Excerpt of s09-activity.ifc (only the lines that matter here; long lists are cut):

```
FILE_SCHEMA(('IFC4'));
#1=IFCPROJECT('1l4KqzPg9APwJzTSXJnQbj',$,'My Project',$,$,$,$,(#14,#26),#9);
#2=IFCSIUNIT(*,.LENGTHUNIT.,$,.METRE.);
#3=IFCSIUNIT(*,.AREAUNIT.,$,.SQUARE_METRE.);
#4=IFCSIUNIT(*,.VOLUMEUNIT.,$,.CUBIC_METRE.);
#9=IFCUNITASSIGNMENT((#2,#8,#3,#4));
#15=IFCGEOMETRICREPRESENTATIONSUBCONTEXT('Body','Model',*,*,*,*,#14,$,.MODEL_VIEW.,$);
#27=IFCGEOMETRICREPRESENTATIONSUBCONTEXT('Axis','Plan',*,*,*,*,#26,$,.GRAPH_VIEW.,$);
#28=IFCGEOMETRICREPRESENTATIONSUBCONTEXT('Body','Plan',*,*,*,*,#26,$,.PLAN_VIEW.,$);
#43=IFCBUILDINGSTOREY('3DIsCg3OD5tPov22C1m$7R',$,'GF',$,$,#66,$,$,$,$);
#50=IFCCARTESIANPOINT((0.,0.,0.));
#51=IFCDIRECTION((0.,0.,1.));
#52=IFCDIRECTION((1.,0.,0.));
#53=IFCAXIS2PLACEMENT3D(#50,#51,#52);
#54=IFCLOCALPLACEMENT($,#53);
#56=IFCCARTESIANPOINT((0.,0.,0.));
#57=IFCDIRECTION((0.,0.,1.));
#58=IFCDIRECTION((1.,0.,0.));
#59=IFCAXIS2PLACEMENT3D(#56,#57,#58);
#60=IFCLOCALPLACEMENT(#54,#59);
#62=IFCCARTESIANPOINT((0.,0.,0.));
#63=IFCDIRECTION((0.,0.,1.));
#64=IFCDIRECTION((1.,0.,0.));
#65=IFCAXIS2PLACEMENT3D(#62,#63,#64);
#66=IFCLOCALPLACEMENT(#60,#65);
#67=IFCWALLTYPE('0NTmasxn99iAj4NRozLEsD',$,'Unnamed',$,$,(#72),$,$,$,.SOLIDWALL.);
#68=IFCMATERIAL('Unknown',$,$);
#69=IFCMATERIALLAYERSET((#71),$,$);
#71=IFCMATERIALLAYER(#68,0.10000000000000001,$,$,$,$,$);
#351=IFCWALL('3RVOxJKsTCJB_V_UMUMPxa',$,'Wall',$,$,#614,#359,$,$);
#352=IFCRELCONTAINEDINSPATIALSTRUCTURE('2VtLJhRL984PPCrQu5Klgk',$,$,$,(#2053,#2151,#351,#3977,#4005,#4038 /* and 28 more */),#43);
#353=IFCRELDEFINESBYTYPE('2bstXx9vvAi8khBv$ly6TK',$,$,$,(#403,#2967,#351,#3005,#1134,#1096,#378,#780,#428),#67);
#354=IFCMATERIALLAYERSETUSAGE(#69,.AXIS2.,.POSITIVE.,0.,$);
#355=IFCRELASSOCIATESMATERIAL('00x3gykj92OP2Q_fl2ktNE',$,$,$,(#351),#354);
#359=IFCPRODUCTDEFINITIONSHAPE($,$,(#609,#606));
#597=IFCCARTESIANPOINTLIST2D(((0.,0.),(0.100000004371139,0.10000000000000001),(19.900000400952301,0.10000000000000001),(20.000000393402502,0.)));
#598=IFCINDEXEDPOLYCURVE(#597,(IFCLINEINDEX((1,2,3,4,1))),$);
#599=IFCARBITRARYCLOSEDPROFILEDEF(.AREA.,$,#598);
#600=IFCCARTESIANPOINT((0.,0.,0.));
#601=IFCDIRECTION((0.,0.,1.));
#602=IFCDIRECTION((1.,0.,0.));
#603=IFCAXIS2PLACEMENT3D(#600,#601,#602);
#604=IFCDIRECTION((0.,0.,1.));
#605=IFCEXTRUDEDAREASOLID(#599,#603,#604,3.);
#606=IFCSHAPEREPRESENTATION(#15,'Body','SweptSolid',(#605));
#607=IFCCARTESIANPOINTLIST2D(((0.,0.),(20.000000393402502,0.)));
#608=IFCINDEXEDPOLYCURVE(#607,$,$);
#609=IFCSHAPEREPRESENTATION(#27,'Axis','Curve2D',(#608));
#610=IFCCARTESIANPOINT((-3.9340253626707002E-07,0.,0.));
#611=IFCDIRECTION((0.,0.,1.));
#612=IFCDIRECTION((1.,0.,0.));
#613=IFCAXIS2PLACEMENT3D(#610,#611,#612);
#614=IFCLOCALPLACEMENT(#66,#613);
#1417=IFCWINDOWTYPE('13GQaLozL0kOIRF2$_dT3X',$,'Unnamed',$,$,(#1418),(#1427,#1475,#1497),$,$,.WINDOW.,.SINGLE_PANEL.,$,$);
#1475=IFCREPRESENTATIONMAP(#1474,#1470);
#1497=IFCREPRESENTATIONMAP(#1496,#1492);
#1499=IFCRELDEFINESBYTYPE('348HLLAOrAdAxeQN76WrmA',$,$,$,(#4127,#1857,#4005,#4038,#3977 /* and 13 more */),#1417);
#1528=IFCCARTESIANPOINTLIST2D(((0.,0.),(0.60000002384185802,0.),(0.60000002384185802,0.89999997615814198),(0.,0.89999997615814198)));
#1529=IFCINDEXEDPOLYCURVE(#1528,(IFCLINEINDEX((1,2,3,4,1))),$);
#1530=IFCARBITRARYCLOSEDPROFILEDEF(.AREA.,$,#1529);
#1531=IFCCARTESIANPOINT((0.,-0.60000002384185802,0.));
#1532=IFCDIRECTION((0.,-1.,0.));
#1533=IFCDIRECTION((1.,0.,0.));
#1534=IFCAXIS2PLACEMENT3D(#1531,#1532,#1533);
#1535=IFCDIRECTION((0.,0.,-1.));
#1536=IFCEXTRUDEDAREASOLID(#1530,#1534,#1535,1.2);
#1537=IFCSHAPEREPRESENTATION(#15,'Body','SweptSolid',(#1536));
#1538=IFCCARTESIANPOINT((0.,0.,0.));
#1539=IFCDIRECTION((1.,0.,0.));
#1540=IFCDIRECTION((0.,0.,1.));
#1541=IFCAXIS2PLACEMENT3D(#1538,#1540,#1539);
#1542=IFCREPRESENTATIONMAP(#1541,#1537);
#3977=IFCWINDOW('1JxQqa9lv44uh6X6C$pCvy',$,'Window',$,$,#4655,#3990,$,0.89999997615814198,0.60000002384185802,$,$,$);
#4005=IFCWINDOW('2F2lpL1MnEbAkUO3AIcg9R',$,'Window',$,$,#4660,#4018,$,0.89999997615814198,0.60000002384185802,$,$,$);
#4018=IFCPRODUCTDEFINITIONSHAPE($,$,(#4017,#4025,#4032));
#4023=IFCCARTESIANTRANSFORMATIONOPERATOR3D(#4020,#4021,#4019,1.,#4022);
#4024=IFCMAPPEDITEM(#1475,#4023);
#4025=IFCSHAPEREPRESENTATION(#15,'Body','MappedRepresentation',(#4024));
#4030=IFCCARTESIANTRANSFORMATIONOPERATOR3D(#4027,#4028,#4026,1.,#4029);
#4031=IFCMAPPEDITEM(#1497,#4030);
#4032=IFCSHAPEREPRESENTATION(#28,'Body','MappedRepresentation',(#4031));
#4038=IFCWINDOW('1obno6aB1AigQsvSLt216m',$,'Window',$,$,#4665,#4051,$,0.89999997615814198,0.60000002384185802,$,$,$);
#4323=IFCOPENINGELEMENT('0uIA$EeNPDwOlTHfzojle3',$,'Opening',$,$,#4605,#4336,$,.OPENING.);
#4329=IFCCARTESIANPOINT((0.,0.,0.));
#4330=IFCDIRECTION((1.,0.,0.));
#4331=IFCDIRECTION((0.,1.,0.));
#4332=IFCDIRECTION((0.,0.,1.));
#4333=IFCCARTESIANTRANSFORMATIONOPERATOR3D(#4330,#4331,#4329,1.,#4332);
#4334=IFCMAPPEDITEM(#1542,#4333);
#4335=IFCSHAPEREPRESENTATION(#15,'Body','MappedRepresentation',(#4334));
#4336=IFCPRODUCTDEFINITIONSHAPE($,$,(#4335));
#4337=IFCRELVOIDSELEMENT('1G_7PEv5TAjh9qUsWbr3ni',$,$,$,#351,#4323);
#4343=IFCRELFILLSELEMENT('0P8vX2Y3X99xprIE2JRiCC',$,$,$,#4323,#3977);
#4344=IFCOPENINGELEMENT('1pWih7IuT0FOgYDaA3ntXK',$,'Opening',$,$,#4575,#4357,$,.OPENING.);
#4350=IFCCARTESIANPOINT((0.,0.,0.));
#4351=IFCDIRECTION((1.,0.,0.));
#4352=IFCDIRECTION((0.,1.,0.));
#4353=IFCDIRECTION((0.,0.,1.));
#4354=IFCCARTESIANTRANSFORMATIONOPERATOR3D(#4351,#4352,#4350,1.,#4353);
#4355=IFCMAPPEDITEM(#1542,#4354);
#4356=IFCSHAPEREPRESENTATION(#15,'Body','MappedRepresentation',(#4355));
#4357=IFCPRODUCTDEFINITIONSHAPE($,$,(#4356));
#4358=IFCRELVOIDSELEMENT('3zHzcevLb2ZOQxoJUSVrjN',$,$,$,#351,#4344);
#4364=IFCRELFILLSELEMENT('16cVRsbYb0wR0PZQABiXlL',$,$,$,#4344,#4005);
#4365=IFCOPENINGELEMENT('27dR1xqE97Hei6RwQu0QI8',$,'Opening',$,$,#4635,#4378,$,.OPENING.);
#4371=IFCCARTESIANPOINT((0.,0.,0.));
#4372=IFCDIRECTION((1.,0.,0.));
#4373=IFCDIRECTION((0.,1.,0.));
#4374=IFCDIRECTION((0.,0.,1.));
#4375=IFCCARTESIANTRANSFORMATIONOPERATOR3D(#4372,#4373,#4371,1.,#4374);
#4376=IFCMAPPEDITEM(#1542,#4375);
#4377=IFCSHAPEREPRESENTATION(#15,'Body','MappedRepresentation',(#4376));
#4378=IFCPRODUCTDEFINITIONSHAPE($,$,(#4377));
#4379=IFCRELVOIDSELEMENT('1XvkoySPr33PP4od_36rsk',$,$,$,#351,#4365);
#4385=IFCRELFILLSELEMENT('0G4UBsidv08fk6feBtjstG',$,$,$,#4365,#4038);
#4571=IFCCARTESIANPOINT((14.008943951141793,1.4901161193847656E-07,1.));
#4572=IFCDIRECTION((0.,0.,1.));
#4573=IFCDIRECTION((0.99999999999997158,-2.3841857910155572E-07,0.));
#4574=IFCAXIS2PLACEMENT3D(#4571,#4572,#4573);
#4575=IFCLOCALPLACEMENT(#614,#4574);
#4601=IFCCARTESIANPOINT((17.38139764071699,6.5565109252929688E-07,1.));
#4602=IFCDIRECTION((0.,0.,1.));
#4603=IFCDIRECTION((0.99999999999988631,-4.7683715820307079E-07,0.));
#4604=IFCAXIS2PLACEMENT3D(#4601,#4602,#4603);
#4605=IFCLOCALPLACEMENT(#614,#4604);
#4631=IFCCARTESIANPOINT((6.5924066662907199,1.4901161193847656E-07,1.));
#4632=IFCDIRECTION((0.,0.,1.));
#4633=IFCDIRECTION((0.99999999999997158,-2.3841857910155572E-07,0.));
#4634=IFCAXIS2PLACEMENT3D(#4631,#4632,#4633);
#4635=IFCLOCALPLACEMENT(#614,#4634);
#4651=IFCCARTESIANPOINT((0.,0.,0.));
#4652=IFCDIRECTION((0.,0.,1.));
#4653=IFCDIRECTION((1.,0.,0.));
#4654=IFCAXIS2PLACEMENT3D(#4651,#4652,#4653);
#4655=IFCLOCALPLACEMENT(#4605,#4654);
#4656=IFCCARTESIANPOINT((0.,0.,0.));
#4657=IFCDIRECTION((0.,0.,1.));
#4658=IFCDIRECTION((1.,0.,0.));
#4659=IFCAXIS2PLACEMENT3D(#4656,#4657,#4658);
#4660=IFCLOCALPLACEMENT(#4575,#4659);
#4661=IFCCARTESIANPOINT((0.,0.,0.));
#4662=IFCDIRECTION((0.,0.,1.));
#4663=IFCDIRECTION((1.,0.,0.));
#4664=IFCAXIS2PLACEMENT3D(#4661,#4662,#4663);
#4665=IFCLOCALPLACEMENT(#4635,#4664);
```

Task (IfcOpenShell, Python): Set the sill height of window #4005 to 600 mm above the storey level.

```python
import numpy as np
import ifcopenshell
import ifcopenshell.api.geometry
import ifcopenshell.geom
import ifcopenshell.util.element
import ifcopenshell.util.placement
import ifcopenshell.util.shape
import ifcopenshell.util.unit

model = ifcopenshell.open("s09-activity.ifc")
unit_scale = ifcopenshell.util.unit.calculate_unit_scale(model)

window = model.by_id(4005)
opening = window.FillsVoids[0].RelatingOpeningElement
storey = ifcopenshell.util.element.get_container(window, ifc_class="IfcBuildingStorey")
level = ifcopenshell.util.placement.get_local_placement(storey.ObjectPlacement)[2, 3]

# The opening's origin need not be at the sill, so measure its lowest point.
shape = ifcopenshell.geom.create_shape(ifcopenshell.geom.settings(), opening)
bottom = ifcopenshell.util.shape.get_shape_bottom_elevation(shape, shape.geometry) / unit_scale
dz = level + 0.6 - bottom

shift = np.array([0.0, 0.0, dz])
# The window is placed relative to its opening, so it follows when the opening moves.
matrix = ifcopenshell.util.placement.get_local_placement(opening.ObjectPlacement)
matrix[:3, 3] += shift
ifcopenshell.api.geometry.edit_object_placement(
    model, product=opening, matrix=matrix, is_si=False, should_transform_children=True
)

print(f"moved by {dz * unit_scale:+.3f} m")

model.write("s09-activity_v2.ifc")
```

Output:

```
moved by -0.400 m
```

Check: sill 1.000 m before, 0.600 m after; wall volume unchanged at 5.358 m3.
